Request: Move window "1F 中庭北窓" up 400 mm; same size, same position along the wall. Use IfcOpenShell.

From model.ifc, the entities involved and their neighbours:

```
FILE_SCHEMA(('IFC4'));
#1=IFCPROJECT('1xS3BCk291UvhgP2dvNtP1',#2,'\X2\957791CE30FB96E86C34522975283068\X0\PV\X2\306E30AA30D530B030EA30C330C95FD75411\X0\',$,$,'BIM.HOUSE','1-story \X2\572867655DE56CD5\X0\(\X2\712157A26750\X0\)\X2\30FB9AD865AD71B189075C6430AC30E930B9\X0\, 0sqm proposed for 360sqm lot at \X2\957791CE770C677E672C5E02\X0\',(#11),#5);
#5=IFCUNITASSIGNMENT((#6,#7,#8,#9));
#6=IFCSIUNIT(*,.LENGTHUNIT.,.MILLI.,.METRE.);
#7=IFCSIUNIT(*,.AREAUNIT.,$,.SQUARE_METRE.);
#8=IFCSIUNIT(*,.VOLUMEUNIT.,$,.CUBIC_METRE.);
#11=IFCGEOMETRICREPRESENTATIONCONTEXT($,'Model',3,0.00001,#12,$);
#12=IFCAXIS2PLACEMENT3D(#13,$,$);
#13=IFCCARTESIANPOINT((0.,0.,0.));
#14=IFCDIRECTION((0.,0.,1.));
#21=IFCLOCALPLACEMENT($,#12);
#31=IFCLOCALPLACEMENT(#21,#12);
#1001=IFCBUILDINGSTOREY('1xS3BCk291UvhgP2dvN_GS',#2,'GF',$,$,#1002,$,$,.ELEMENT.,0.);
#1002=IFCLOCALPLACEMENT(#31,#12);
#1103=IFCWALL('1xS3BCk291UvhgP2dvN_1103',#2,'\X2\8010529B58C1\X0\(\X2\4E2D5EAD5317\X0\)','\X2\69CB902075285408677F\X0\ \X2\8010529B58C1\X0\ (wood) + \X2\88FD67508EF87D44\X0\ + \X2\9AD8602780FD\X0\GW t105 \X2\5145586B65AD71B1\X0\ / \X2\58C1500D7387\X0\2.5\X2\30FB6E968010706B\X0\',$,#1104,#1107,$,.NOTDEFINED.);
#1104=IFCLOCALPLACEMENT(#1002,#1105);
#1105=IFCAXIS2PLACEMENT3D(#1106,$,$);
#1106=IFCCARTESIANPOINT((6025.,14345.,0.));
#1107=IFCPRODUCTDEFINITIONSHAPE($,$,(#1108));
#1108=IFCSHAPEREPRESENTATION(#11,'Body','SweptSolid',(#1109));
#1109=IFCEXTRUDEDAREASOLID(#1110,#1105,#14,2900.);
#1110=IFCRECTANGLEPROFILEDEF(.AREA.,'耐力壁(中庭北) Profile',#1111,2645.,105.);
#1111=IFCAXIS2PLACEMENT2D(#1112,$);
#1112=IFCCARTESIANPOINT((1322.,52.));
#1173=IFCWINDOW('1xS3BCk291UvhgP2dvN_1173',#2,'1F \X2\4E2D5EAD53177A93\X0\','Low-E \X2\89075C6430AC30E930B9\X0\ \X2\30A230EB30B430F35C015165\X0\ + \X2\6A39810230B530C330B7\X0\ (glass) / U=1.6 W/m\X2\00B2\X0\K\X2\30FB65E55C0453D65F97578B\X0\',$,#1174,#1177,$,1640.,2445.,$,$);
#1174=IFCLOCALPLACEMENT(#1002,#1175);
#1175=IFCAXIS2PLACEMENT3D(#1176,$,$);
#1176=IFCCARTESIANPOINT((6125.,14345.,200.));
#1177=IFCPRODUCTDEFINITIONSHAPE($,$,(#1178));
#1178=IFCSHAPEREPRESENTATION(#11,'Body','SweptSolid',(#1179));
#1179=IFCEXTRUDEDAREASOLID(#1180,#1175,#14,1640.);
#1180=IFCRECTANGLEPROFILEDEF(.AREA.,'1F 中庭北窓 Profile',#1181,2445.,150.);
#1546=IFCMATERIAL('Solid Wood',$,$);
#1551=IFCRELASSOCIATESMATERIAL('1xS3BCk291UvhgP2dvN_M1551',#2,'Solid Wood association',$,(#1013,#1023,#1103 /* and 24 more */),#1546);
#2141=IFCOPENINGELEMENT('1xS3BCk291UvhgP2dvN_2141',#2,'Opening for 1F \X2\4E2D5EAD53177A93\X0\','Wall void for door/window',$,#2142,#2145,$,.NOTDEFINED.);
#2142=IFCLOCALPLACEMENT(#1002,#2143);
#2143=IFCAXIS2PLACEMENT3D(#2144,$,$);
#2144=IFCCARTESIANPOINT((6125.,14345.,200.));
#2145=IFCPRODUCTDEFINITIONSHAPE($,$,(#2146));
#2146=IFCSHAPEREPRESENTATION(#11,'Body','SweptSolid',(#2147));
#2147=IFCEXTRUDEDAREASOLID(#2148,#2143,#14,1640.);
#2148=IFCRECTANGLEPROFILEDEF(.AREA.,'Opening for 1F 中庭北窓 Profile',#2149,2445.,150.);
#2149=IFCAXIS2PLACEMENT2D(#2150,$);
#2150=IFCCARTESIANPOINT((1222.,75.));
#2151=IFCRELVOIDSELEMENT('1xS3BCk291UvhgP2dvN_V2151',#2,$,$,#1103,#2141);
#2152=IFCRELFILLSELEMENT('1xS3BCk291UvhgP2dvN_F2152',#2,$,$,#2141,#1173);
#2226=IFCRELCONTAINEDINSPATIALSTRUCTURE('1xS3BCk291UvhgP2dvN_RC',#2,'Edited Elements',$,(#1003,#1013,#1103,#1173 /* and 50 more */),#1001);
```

```python
import numpy as np
import ifcopenshell
import ifcopenshell.api.geometry
import ifcopenshell.util.placement
import ifcopenshell.util.unit

model = ifcopenshell.open("model.ifc")
unit_scale = ifcopenshell.util.unit.calculate_unit_scale(model)

window = model.by_id(1173)
opening = window.FillsVoids[0].RelatingOpeningElement
dz = 0.4 / unit_scale

shift = np.array([0.0, 0.0, dz])
# The window is not placed relative to its opening, so move both.
for product in (opening, window):
    matrix = ifcopenshell.util.placement.get_local_placement(product.ObjectPlacement)
    matrix[:3, 3] += shift
    ifcopenshell.api.geometry.edit_object_placement(model, product=product, matrix=matrix, is_si=False)

print(f"moved by {dz * unit_scale:+.3f} m")

model.write("model_v2.ifc")
```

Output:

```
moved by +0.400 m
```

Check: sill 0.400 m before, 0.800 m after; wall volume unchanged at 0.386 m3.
